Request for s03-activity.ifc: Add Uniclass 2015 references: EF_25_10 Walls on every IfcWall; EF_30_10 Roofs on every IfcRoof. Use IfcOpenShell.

First a look at what the model holds.

```python
import ifcopenshell

model = ifcopenshell.open("s03-activity.ifc")
print(model.schema)
print("classifications:", [c.Name for c in model.by_type("IfcClassification")])
for ifc_class in ("IfcDoor", "IfcRoof", "IfcStair", "IfcWall", "IfcWindow"):
    print(ifc_class, len(model.by_type(ifc_class)))
```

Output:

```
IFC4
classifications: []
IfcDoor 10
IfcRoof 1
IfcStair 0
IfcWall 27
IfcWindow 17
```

```python
import ifcopenshell
import ifcopenshell.api.classification

model = ifcopenshell.open("s03-activity.ifc")

system = ifcopenshell.api.classification.add_classification(model, classification="Uniclass 2015")

codes = {
    "IfcWall": ("EF_25_10", "Walls"),
    "IfcRoof": ("EF_30_10", "Roofs"),
}
for ifc_class, (code, name) in codes.items():
    products = model.by_type(ifc_class)
    ifcopenshell.api.classification.add_reference(
        model, products=products, classification=system, identification=code, name=name
    )
    print(code, len(products))

model.write("s03-activity-out.ifc")
```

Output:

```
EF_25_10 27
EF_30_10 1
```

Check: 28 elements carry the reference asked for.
